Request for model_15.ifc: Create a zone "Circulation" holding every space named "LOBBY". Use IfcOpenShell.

First a look at what the model holds.

```python
import ifcopenshell

model = ifcopenshell.open("model_15.ifc")
print(model.schema)
seen = {}
for space in model.by_type("IfcSpace"):
    seen[space.LongName] = seen.get(space.LongName, 0) + 1
for name, count in sorted(seen.items(), key=str):
    print(count, "x", name)
print("zones:", [z.Name for z in model.by_type("IfcZone")][:20])
```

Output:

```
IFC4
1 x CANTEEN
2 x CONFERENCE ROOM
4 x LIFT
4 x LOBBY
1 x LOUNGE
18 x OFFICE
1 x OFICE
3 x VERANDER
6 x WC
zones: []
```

```python
import ifcopenshell
import ifcopenshell.api.group
import ifcopenshell.api.root

model = ifcopenshell.open("model_15.ifc")

names = {"LOBBY"}
spaces = [s for s in model.by_type("IfcSpace") if s.LongName in names]

zone = ifcopenshell.api.root.create_entity(model, ifc_class="IfcZone", name="Circulation")
ifcopenshell.api.group.assign_group(model, products=spaces, group=zone)
print(len(spaces), "spaces in", zone.Name)

model.write("model_15-out.ifc")
```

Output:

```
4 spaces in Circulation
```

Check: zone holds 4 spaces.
